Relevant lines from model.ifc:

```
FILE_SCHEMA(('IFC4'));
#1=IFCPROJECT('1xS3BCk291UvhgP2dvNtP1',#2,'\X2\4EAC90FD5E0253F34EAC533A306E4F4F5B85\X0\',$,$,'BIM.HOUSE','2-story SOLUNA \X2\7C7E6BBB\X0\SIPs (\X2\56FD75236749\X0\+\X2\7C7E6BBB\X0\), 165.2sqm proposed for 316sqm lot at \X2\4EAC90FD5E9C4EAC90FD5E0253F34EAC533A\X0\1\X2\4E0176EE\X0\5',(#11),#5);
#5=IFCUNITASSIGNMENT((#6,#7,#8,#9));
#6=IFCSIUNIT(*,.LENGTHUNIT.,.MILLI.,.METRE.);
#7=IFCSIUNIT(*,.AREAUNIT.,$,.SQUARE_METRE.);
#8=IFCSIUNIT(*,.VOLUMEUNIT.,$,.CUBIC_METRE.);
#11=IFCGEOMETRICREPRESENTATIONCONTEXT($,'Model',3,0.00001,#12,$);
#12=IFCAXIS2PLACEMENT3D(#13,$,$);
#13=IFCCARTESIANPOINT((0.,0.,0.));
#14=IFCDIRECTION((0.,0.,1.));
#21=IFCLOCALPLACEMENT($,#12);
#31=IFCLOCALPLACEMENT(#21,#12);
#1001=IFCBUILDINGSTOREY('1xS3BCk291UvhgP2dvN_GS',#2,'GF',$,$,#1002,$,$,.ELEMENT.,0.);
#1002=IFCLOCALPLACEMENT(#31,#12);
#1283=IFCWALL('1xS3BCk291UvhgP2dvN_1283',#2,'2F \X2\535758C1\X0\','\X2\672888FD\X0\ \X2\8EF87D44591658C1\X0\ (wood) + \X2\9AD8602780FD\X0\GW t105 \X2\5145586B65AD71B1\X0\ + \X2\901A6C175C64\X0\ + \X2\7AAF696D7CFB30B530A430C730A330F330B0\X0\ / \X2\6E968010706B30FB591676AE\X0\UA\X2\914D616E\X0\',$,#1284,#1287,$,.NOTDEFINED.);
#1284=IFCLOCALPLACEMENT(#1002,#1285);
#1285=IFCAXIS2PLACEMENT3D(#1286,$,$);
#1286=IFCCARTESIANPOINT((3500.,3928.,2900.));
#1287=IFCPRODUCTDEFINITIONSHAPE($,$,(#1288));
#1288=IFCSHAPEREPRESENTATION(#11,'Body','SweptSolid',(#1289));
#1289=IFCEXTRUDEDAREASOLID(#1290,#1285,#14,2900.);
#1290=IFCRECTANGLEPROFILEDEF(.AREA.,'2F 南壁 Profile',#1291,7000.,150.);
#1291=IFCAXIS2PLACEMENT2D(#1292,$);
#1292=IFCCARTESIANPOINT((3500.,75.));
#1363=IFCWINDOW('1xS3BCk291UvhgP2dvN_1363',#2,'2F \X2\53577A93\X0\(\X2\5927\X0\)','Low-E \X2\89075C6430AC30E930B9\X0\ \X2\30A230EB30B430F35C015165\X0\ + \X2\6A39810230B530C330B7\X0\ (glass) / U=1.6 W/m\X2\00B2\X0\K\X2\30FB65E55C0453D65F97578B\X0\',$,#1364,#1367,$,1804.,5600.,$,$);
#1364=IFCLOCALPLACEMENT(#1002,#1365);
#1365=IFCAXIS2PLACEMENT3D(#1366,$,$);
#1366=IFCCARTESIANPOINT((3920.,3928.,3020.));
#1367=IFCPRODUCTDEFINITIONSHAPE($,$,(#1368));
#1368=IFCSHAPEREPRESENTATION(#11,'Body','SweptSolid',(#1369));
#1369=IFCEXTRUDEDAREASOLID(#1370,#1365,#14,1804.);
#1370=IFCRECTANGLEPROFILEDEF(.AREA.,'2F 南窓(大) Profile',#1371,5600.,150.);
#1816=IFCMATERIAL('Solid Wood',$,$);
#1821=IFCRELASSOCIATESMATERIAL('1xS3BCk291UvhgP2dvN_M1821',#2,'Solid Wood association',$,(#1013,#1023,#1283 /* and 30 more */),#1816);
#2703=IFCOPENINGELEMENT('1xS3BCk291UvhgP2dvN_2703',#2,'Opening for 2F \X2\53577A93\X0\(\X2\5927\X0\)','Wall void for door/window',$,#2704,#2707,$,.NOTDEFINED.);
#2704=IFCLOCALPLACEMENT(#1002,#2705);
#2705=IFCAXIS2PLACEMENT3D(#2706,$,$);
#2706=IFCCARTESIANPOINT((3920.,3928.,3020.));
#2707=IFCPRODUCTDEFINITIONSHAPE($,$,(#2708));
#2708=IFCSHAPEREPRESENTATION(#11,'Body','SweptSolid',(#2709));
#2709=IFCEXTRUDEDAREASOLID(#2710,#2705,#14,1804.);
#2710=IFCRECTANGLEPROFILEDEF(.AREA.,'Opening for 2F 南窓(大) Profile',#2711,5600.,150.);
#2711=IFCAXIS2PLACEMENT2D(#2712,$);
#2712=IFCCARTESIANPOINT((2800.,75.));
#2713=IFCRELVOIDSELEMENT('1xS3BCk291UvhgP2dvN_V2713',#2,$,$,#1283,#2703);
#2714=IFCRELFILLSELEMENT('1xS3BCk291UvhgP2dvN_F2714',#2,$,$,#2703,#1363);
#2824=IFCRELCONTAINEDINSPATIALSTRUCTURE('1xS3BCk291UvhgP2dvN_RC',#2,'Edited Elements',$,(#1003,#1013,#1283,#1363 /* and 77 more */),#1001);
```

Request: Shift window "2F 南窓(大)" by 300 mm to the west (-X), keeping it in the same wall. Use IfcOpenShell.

```python
import ifcopenshell
import ifcopenshell.api.geometry
import ifcopenshell.util.placement

model = ifcopenshell.open("model.ifc")

window = model.by_guid("1xS3BCk291UvhgP2dvN_1363")
opening = window.FillsVoids[0].RelatingOpeningElement
wall = opening.VoidsElements[0].RelatingBuildingElement

wall_matrix = ifcopenshell.util.placement.get_local_placement(wall.ObjectPlacement)
shift = wall_matrix[:3, 0] * -300.0
before = ifcopenshell.util.placement.get_local_placement(window.ObjectPlacement)[:3, 3].copy()

# The window is not placed relative to its opening, so move both.
for product in (opening, window):
    matrix = ifcopenshell.util.placement.get_local_placement(product.ObjectPlacement)
    matrix[:3, 3] += shift
    ifcopenshell.api.geometry.edit_object_placement(model, product=product, matrix=matrix, is_si=False)

after = ifcopenshell.util.placement.get_local_placement(window.ObjectPlacement)[:3, 3]
print("window moved by", (after - before).round(3) + 0.0)

model.write("model_edited.ifc")
```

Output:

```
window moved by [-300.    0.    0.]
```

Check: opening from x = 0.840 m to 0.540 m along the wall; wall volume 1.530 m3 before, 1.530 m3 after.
